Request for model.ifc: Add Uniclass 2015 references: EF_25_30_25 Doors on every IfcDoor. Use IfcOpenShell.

First a look at what the model holds.

```python
import ifcopenshell

model = ifcopenshell.open("model.ifc")
print(model.schema)
print("classifications:", [c.Name for c in model.by_type("IfcClassification")])
for ifc_class in ("IfcDoor", "IfcRoof", "IfcStair", "IfcWall", "IfcWindow"):
    print(ifc_class, len(model.by_type(ifc_class)))
```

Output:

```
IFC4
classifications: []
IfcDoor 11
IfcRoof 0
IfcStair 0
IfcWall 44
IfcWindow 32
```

```python
import ifcopenshell
import ifcopenshell.api.classification

model = ifcopenshell.open("model.ifc")

system = ifcopenshell.api.classification.add_classification(model, classification="Uniclass 2015")

codes = {
    "IfcDoor": ("EF_25_30_25", "Doors"),
}
for ifc_class, (code, name) in codes.items():
    products = model.by_type(ifc_class)
    ifcopenshell.api.classification.add_reference(
        model, products=products, classification=system, identification=code, name=name
    )
    print(code, len(products))

model.write("model_edited.ifc")
```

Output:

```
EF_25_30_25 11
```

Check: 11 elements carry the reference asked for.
